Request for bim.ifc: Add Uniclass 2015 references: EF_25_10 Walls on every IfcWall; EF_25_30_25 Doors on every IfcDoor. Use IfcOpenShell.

First a look at what the model holds.

```python
import ifcopenshell

model = ifcopenshell.open("bim.ifc")
print(model.schema)
print("classifications:", [c.Name for c in model.by_type("IfcClassification")])
for ifc_class in ("IfcDoor", "IfcRoof", "IfcStair", "IfcWall", "IfcWindow"):
    print(ifc_class, len(model.by_type(ifc_class)))
```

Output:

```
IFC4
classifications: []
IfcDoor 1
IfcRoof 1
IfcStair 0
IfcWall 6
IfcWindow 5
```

```python
import ifcopenshell
import ifcopenshell.api.classification

model = ifcopenshell.open("bim.ifc")

system = ifcopenshell.api.classification.add_classification(model, classification="Uniclass 2015")

codes = {
    "IfcWall": ("EF_25_10", "Walls"),
    "IfcDoor": ("EF_25_30_25", "Doors"),
}
for ifc_class, (code, name) in codes.items():
    products = model.by_type(ifc_class)
    ifcopenshell.api.classification.add_reference(
        model, products=products, classification=system, identification=code, name=name
    )
    print(code, len(products))

model.write("bim_updated.ifc")
```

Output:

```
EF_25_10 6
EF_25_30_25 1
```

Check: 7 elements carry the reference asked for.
